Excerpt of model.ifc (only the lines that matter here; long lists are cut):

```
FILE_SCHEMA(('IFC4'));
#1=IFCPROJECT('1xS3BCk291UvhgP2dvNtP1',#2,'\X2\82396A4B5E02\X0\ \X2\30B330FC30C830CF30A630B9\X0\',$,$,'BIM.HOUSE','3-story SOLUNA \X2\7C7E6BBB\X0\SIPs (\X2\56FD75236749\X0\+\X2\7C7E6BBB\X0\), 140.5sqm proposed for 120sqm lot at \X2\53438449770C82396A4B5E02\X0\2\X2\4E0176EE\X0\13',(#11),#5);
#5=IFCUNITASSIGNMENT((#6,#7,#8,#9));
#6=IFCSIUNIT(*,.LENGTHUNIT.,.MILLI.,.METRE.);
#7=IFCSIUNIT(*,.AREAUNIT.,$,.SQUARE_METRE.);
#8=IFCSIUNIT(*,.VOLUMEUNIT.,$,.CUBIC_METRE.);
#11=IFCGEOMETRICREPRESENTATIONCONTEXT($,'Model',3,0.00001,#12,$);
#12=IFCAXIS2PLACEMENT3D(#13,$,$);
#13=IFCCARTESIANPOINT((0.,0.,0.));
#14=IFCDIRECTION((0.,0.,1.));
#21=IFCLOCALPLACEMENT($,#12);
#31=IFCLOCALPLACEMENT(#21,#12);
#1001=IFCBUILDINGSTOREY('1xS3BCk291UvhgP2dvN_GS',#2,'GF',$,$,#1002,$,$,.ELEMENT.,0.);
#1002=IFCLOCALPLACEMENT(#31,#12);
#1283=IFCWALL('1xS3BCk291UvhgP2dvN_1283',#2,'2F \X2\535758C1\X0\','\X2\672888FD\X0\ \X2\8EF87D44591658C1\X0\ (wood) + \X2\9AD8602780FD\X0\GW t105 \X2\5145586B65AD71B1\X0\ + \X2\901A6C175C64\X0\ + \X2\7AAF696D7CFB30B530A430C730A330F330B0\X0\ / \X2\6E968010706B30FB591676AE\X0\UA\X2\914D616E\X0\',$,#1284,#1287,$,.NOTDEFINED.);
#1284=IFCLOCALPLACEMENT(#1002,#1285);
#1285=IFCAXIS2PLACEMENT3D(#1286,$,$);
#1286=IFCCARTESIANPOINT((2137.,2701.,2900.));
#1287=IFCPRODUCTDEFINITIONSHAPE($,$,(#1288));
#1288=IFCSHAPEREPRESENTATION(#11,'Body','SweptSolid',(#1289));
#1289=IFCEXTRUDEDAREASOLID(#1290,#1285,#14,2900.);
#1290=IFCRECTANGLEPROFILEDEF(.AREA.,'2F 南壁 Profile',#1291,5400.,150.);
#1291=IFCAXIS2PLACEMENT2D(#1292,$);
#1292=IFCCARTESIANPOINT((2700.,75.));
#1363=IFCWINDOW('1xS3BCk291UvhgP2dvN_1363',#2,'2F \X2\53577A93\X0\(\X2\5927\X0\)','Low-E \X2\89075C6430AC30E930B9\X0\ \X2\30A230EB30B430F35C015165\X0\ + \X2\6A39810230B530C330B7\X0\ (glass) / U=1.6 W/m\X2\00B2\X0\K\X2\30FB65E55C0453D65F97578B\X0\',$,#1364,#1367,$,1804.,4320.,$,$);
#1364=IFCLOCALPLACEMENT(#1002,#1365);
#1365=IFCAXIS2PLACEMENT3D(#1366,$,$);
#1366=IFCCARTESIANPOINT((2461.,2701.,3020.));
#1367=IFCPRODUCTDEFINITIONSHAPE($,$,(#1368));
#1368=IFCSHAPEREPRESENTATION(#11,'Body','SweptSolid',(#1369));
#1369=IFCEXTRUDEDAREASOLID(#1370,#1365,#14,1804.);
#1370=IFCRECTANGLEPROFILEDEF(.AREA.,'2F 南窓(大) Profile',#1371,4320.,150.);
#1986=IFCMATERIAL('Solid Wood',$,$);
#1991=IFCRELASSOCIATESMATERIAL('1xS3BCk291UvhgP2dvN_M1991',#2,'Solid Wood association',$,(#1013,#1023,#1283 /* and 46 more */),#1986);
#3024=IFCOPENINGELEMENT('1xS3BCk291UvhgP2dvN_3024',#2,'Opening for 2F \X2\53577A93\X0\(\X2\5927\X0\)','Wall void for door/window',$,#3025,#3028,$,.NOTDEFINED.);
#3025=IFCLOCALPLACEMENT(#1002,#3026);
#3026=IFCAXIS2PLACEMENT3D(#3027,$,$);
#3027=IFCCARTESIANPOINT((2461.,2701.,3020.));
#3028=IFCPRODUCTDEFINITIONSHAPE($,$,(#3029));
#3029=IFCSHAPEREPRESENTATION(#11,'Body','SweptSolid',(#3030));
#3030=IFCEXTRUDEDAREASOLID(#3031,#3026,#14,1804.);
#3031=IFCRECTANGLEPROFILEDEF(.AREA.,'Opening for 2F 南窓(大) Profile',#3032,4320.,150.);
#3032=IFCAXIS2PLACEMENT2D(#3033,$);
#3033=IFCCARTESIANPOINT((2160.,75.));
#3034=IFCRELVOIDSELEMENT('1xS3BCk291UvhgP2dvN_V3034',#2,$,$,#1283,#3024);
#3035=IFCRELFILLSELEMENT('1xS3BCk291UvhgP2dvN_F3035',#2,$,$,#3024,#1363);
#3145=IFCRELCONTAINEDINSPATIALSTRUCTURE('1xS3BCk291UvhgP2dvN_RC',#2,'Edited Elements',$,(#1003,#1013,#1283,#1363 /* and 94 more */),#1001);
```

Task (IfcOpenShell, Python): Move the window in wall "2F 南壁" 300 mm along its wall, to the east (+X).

```python
import ifcopenshell
import ifcopenshell.api.geometry
import ifcopenshell.util.placement

model = ifcopenshell.open("model.ifc")

window = model.by_guid("1xS3BCk291UvhgP2dvN_1363")
opening = window.FillsVoids[0].RelatingOpeningElement
wall = opening.VoidsElements[0].RelatingBuildingElement

wall_matrix = ifcopenshell.util.placement.get_local_placement(wall.ObjectPlacement)
shift = wall_matrix[:3, 0] * 300.0
before = ifcopenshell.util.placement.get_local_placement(window.ObjectPlacement)[:3, 3].copy()

# The window is not placed relative to its opening, so move both.
for product in (opening, window):
    matrix = ifcopenshell.util.placement.get_local_placement(product.ObjectPlacement)
    matrix[:3, 3] += shift
    ifcopenshell.api.geometry.edit_object_placement(model, product=product, matrix=matrix, is_si=False)

after = ifcopenshell.util.placement.get_local_placement(window.ObjectPlacement)[:3, 3]
print("window moved by", (after - before).round(3) + 0.0)

model.write("model-out.ifc")
```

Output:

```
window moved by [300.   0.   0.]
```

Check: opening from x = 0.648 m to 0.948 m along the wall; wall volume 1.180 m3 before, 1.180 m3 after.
